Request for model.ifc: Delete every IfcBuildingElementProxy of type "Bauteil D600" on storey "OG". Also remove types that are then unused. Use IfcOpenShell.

First a look at what the model holds.

```python
import ifcopenshell
import ifcopenshell.util.element

model = ifcopenshell.open("model.ifc")
print(model.schema)
storey = next(s for s in model.by_type("IfcBuildingStorey") if s.Name == "OG")
proxies = [e for e in ifcopenshell.util.element.get_decomposition(storey) if e.is_a("IfcBuildingElementProxy")]
seen = {}
for e in proxies:
    element_type = ifcopenshell.util.element.get_type(e)
    name = element_type.Name if element_type not in (None, e) else None
    seen[name] = seen.get(name, 0) + 1
for name, count in sorted(seen.items(), key=str):
    print(count, "x", name)
```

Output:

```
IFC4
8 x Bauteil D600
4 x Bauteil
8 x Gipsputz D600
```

```python
import ifcopenshell
import ifcopenshell.api.root
import ifcopenshell.util.element

model = ifcopenshell.open("model.ifc")

storey = next(s for s in model.by_type("IfcBuildingStorey") if s.Name == "OG")
proxies = [e for e in ifcopenshell.util.element.get_decomposition(storey) if e.is_a("IfcBuildingElementProxy")]
targets = [e for e in proxies if (t := ifcopenshell.util.element.get_type(e)) not in (None, e) and t.Name == "Bauteil D600"]
types = {ifcopenshell.util.element.get_type(e) for e in targets} - {None, *targets}

for e in targets:
    ifcopenshell.api.root.remove_product(model, product=e)
print(len(targets), "removed")

unused = [t for t in types if not ifcopenshell.util.element.get_types(t)]
for t in unused:
    ifcopenshell.api.root.remove_product(model, product=t)
print(len(unused), "unused types removed")

model.write("model_v2.ifc")
```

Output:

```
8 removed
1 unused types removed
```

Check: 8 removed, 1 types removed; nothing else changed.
